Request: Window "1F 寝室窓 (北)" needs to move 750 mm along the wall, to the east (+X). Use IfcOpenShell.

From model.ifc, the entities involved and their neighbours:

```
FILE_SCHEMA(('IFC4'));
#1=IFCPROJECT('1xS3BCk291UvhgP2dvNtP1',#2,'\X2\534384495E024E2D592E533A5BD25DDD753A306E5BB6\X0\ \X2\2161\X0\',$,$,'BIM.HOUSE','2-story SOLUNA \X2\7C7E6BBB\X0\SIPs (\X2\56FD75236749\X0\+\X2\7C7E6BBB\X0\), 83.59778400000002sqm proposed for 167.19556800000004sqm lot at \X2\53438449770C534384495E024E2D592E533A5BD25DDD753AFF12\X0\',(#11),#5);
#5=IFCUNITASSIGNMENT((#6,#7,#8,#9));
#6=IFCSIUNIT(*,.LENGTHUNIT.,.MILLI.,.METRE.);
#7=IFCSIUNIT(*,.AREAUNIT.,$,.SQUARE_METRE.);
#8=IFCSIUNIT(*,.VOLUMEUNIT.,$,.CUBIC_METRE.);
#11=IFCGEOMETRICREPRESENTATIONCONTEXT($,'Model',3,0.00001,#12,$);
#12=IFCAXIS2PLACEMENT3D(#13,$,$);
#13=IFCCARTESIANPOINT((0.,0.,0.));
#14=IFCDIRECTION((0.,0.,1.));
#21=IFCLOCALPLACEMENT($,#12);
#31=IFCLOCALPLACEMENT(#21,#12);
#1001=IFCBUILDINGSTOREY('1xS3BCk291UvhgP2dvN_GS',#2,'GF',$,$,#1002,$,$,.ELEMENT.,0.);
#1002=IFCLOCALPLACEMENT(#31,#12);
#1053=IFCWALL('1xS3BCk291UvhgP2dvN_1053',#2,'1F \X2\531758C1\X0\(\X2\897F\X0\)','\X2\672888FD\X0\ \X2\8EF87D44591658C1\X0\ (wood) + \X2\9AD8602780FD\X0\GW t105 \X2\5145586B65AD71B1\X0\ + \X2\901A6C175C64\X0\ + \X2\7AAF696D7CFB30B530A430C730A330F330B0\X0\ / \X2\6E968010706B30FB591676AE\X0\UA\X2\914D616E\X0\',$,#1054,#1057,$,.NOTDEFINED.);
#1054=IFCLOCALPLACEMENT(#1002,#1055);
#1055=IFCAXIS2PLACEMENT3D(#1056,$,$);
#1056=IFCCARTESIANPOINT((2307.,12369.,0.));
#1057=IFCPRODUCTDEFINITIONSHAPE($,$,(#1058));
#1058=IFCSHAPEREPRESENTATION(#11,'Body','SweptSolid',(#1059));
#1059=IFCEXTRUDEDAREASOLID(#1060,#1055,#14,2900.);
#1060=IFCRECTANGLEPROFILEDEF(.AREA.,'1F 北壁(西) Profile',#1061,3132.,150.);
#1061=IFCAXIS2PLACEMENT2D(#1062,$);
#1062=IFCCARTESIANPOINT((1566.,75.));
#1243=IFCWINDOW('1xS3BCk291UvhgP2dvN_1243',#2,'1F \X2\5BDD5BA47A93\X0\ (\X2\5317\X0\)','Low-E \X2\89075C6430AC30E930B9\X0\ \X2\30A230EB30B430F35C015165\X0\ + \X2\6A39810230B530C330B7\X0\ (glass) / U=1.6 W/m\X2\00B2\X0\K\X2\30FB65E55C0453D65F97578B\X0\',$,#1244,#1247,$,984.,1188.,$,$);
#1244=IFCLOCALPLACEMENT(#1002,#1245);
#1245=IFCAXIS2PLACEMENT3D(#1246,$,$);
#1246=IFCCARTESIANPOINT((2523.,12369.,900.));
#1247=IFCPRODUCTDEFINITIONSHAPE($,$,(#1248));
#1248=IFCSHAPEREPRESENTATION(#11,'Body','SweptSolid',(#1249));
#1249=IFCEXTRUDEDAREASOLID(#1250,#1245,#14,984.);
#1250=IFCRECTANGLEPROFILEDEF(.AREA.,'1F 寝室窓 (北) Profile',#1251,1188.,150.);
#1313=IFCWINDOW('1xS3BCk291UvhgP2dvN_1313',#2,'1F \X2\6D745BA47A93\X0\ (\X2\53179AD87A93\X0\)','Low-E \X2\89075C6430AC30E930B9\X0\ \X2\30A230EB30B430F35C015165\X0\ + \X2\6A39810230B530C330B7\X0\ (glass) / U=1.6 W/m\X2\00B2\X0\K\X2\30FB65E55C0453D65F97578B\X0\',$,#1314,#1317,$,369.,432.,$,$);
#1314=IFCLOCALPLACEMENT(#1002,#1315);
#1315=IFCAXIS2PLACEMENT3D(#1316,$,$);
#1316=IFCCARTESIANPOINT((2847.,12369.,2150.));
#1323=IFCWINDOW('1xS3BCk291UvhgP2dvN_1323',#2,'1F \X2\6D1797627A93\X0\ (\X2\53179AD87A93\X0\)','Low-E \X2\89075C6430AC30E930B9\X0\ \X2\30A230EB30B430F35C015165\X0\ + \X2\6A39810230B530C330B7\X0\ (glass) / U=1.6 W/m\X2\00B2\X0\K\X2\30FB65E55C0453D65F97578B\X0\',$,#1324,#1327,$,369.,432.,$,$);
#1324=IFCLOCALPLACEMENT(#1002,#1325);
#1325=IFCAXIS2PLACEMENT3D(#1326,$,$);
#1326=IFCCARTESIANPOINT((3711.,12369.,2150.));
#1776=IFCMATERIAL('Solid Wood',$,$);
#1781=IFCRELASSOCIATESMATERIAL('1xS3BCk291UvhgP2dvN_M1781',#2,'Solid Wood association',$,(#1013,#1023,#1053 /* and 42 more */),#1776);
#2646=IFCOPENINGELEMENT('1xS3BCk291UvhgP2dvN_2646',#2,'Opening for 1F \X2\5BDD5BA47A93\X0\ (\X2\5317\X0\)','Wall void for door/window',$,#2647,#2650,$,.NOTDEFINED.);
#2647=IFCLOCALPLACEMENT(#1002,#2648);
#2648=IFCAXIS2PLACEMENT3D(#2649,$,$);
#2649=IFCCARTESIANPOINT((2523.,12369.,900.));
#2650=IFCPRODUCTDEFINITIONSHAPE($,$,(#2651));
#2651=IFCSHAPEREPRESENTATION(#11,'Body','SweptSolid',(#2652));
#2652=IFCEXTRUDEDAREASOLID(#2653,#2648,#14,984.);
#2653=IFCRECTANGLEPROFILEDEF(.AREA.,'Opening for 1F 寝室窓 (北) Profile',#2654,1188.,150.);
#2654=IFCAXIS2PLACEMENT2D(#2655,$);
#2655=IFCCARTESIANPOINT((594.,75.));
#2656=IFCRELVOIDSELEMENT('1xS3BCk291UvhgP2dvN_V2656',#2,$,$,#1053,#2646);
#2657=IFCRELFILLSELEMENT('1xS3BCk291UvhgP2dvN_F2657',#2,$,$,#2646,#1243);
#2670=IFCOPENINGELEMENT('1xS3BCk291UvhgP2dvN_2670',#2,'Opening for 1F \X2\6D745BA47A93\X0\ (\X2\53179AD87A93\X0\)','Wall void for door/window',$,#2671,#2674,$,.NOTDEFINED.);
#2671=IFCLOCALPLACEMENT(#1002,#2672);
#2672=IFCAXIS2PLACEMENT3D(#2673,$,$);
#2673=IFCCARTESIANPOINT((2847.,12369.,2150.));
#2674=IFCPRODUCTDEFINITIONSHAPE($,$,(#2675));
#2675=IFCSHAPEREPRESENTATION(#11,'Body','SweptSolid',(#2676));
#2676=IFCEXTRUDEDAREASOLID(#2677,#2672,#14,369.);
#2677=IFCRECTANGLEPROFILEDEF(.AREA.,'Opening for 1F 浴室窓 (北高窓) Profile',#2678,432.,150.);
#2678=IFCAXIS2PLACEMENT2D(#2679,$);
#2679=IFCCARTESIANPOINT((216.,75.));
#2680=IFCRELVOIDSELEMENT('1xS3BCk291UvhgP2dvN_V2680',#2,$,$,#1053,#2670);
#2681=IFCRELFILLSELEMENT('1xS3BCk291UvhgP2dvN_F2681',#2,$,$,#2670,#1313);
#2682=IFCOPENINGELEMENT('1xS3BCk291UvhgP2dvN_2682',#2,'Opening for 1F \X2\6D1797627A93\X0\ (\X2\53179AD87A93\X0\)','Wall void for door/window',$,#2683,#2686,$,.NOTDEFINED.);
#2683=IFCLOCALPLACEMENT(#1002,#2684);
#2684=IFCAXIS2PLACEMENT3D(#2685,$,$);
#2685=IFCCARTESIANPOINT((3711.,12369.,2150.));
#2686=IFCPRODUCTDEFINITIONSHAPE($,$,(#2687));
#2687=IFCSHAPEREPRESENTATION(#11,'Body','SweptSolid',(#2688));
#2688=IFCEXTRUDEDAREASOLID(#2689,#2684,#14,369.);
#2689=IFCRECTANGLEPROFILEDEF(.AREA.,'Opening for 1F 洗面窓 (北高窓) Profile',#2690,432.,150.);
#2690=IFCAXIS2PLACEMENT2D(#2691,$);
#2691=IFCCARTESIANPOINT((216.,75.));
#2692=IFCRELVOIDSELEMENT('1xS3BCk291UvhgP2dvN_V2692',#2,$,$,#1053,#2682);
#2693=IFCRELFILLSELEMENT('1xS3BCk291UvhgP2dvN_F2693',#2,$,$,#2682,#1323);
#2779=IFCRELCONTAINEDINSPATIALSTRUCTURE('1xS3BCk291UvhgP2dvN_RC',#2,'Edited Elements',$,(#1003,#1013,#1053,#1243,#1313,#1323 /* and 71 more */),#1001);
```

```python
import ifcopenshell
import ifcopenshell.api.geometry
import ifcopenshell.util.placement
import ifcopenshell.util.unit

model = ifcopenshell.open("model.ifc")
unit_scale = ifcopenshell.util.unit.calculate_unit_scale(model)

window = model.by_guid("1xS3BCk291UvhgP2dvN_1243")
opening = window.FillsVoids[0].RelatingOpeningElement
wall = opening.VoidsElements[0].RelatingBuildingElement

wall_matrix = ifcopenshell.util.placement.get_local_placement(wall.ObjectPlacement)
shift = wall_matrix[:3, 0] * 0.75 / unit_scale
before = ifcopenshell.util.placement.get_local_placement(window.ObjectPlacement)[:3, 3].copy()

# The window is not placed relative to its opening, so move both.
for product in (opening, window):
    matrix = ifcopenshell.util.placement.get_local_placement(product.ObjectPlacement)
    matrix[:3, 3] += shift
    ifcopenshell.api.geometry.edit_object_placement(model, product=product, matrix=matrix, is_si=False)

after = ifcopenshell.util.placement.get_local_placement(window.ObjectPlacement)[:3, 3]
print("window moved by", (after - before).round(3) + 0.0)

model.write("model_updated.ifc")
```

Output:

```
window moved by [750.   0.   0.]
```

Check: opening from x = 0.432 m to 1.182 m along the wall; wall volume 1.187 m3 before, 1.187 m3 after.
